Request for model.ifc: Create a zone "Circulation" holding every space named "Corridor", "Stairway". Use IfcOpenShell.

First a look at what the model holds.

```python
import ifcopenshell

model = ifcopenshell.open("model.ifc")
print(model.schema)
seen = {}
for space in model.by_type("IfcSpace"):
    seen[space.LongName] = seen.get(space.LongName, 0) + 1
for name, count in sorted(seen.items(), key=str):
    print(count, "x", name)
print("zones:", [z.Name for z in model.by_type("IfcZone")][:20])
```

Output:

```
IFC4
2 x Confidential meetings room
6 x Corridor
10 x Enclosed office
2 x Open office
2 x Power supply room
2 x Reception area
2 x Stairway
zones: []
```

```python
import ifcopenshell
import ifcopenshell.api.group
import ifcopenshell.api.root

model = ifcopenshell.open("model.ifc")

names = {"Corridor", "Stairway"}
spaces = [s for s in model.by_type("IfcSpace") if s.LongName in names]

zone = ifcopenshell.api.root.create_entity(model, ifc_class="IfcZone", name="Circulation")
ifcopenshell.api.group.assign_group(model, products=spaces, group=zone)
print(len(spaces), "spaces in", zone.Name)

model.write("model-out.ifc")
```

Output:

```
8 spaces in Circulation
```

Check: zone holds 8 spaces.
